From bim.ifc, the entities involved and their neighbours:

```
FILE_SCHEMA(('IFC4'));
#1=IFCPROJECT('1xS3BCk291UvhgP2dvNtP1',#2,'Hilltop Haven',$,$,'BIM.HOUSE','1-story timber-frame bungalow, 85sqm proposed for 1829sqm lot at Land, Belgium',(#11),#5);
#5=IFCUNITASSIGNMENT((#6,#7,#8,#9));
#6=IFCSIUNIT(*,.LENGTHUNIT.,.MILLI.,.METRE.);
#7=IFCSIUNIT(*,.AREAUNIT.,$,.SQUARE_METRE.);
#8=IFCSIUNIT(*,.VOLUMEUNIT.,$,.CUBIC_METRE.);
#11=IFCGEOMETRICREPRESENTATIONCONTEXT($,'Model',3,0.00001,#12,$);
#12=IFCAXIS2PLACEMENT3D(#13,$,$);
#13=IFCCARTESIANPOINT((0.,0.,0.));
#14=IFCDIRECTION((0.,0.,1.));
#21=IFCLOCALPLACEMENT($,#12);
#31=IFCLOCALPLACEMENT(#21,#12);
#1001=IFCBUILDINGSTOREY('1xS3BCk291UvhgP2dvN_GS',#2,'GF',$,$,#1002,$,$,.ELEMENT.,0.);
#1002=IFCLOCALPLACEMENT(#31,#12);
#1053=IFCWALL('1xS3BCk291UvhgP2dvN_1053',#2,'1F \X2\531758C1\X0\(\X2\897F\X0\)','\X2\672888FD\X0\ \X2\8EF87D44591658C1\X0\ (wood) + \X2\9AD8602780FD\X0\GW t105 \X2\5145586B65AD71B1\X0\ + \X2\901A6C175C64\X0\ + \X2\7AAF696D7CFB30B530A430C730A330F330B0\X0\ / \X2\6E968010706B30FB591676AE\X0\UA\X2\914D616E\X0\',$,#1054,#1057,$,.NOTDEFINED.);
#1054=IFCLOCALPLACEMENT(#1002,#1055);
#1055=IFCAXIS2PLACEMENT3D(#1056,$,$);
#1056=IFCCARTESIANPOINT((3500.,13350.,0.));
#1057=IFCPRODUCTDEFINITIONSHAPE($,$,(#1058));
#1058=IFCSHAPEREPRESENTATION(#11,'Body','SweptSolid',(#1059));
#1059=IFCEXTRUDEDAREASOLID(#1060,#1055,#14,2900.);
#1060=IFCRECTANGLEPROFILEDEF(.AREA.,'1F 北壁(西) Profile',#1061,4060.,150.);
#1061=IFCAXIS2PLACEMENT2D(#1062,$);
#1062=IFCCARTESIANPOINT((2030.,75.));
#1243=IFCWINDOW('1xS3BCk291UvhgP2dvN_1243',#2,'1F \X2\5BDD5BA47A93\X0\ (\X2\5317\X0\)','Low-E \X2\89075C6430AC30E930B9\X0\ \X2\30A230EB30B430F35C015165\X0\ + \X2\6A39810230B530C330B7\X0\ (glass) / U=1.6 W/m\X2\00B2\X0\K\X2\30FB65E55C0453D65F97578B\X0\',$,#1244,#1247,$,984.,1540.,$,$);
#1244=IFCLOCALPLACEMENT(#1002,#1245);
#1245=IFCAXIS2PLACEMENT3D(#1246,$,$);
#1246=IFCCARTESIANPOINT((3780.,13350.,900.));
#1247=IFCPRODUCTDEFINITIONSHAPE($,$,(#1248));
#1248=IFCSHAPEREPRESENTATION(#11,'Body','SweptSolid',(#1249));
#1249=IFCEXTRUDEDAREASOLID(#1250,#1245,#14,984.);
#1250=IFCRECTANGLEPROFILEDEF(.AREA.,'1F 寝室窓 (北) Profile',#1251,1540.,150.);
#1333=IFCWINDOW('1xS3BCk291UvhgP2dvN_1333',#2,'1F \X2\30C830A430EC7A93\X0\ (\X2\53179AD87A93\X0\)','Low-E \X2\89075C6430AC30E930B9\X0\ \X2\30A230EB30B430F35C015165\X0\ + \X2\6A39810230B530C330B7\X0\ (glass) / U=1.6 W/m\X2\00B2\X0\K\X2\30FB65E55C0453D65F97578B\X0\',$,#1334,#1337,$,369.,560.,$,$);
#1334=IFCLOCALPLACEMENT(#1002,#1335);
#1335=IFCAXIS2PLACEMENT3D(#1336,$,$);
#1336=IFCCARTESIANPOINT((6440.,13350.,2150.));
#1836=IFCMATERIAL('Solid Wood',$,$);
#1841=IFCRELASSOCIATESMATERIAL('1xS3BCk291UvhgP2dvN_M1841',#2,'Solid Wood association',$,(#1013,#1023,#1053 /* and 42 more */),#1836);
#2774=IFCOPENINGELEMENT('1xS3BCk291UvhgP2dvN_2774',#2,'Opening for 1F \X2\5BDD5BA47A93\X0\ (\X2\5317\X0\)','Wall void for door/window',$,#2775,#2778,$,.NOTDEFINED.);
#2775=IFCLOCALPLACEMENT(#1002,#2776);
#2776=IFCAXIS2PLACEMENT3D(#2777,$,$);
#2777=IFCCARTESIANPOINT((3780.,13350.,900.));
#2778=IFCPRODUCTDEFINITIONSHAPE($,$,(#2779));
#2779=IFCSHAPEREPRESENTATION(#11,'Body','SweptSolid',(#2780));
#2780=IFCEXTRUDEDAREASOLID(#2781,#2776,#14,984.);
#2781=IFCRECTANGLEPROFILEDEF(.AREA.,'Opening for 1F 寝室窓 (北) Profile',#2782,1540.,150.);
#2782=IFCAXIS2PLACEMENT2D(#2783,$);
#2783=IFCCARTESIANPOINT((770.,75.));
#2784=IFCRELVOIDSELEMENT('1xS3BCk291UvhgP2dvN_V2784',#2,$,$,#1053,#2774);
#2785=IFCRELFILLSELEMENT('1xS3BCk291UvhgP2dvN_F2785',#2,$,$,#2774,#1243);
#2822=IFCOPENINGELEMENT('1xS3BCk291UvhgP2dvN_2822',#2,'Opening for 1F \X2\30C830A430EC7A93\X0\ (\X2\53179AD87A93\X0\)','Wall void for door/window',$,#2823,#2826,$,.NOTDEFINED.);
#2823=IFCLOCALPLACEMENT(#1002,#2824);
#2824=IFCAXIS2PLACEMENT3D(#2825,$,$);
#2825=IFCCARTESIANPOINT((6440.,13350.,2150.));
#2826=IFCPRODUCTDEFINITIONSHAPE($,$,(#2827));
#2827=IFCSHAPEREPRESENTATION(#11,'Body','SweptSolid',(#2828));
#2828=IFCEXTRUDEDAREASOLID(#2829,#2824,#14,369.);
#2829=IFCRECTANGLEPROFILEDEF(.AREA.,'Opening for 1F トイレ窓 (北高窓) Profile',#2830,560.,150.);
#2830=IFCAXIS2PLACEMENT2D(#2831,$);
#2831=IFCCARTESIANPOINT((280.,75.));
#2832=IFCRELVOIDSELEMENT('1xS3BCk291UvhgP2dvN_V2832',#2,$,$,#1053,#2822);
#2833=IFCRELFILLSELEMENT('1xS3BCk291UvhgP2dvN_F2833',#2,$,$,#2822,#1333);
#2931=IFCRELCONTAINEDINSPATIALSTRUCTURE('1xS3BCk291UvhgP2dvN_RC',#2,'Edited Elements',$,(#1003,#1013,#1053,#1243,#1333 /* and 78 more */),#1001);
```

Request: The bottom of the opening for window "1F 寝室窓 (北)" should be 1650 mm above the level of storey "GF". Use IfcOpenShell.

```python
import numpy as np
import ifcopenshell
import ifcopenshell.api.geometry
import ifcopenshell.geom
import ifcopenshell.util.element
import ifcopenshell.util.placement
import ifcopenshell.util.shape
import ifcopenshell.util.unit

model = ifcopenshell.open("bim.ifc")
unit_scale = ifcopenshell.util.unit.calculate_unit_scale(model)

window = model.by_guid("1xS3BCk291UvhgP2dvN_1243")
opening = window.FillsVoids[0].RelatingOpeningElement
storey = ifcopenshell.util.element.get_container(window, ifc_class="IfcBuildingStorey")
level = ifcopenshell.util.placement.get_local_placement(storey.ObjectPlacement)[2, 3]

# The opening's origin need not be at the sill, so measure its lowest point.
shape = ifcopenshell.geom.create_shape(ifcopenshell.geom.settings(), opening)
bottom = ifcopenshell.util.shape.get_shape_bottom_elevation(shape, shape.geometry) / unit_scale
dz = level + 1650.0 - bottom

shift = np.array([0.0, 0.0, dz])
# The window is not placed relative to its opening, so move both.
for product in (opening, window):
    matrix = ifcopenshell.util.placement.get_local_placement(product.ObjectPlacement)
    matrix[:3, 3] += shift
    ifcopenshell.api.geometry.edit_object_placement(model, product=product, matrix=matrix, is_si=False)

print(f"moved by {dz * unit_scale:+.3f} m")

model.write("bim_edited.ifc")
```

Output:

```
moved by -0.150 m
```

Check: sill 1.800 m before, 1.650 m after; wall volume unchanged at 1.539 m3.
